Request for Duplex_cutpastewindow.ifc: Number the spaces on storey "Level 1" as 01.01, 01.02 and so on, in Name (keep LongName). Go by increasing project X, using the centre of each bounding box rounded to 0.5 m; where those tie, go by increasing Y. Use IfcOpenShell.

First a look at what the model holds.

```python
import ifcopenshell
import ifcopenshell.util.element
import ifcopenshell.util.placement

model = ifcopenshell.open("Duplex_cutpastewindow.ifc")
print(model.schema)
storey = next(s for s in model.by_type("IfcBuildingStorey") if s.Name == "Level 1")
spaces = [e for e in ifcopenshell.util.element.get_decomposition(storey) if e.is_a("IfcSpace")]
for e in sorted(spaces, key=lambda e: e.id()):
    origin = ifcopenshell.util.placement.get_local_placement(e.ObjectPlacement)[:3, 3]
    print(e.id(), e.Name, e.LongName, origin.round(2) + 0.0, sep=" | ")
```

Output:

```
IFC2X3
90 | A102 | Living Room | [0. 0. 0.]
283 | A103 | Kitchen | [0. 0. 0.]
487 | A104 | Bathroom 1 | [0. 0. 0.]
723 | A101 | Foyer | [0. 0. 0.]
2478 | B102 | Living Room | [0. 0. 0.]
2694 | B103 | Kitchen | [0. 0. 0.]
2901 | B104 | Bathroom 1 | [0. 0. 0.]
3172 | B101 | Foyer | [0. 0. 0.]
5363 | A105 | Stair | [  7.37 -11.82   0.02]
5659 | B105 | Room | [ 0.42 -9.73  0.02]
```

```python
import ifcopenshell
import ifcopenshell.geom
import ifcopenshell.util.element
import ifcopenshell.util.shape

model = ifcopenshell.open("Duplex_cutpastewindow.ifc")
settings = ifcopenshell.geom.settings()
settings.set("use-world-coords", True)


def centre(element):
    shape = ifcopenshell.geom.create_shape(settings, element)
    return ifcopenshell.util.shape.get_bbox_centroid(shape.geometry)


storey = next(s for s in model.by_type("IfcBuildingStorey") if s.Name == "Level 1")
spaces = [e for e in ifcopenshell.util.element.get_decomposition(storey) if e.is_a("IfcSpace")]

# Insertion points can sit at a corner or the storey origin, so sort by the geometry (in metres).
centres = {e: centre(e) for e in spaces}
spaces.sort(key=lambda e: (round(centres[e][0] / 0.5), centres[e][1]))

for i, e in enumerate(spaces, start=1):
    number = f"01.{i:02d}"
    e.Name = number
    print(e.id(), number)

model.write("Duplex_cutpastewindow_edited.ifc")
```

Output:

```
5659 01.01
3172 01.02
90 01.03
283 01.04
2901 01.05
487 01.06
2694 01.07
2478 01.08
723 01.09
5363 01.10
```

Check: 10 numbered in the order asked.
